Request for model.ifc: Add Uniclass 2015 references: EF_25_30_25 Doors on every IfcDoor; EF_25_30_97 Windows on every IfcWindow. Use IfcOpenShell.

First a look at what the model holds.

```python
import ifcopenshell

model = ifcopenshell.open("model.ifc")
print(model.schema)
print("classifications:", [c.Name for c in model.by_type("IfcClassification")])
for ifc_class in ("IfcDoor", "IfcRoof", "IfcStair", "IfcWall", "IfcWindow"):
    print(ifc_class, len(model.by_type(ifc_class)))
```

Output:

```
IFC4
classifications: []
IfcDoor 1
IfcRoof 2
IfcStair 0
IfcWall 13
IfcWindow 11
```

```python
import ifcopenshell
import ifcopenshell.api.classification

model = ifcopenshell.open("model.ifc")

system = ifcopenshell.api.classification.add_classification(model, classification="Uniclass 2015")

codes = {
    "IfcDoor": ("EF_25_30_25", "Doors"),
    "IfcWindow": ("EF_25_30_97", "Windows"),
}
for ifc_class, (code, name) in codes.items():
    products = model.by_type(ifc_class)
    ifcopenshell.api.classification.add_reference(
        model, products=products, classification=system, identification=code, name=name
    )
    print(code, len(products))

model.write("model_updated.ifc")
```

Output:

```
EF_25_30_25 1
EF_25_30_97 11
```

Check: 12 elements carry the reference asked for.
